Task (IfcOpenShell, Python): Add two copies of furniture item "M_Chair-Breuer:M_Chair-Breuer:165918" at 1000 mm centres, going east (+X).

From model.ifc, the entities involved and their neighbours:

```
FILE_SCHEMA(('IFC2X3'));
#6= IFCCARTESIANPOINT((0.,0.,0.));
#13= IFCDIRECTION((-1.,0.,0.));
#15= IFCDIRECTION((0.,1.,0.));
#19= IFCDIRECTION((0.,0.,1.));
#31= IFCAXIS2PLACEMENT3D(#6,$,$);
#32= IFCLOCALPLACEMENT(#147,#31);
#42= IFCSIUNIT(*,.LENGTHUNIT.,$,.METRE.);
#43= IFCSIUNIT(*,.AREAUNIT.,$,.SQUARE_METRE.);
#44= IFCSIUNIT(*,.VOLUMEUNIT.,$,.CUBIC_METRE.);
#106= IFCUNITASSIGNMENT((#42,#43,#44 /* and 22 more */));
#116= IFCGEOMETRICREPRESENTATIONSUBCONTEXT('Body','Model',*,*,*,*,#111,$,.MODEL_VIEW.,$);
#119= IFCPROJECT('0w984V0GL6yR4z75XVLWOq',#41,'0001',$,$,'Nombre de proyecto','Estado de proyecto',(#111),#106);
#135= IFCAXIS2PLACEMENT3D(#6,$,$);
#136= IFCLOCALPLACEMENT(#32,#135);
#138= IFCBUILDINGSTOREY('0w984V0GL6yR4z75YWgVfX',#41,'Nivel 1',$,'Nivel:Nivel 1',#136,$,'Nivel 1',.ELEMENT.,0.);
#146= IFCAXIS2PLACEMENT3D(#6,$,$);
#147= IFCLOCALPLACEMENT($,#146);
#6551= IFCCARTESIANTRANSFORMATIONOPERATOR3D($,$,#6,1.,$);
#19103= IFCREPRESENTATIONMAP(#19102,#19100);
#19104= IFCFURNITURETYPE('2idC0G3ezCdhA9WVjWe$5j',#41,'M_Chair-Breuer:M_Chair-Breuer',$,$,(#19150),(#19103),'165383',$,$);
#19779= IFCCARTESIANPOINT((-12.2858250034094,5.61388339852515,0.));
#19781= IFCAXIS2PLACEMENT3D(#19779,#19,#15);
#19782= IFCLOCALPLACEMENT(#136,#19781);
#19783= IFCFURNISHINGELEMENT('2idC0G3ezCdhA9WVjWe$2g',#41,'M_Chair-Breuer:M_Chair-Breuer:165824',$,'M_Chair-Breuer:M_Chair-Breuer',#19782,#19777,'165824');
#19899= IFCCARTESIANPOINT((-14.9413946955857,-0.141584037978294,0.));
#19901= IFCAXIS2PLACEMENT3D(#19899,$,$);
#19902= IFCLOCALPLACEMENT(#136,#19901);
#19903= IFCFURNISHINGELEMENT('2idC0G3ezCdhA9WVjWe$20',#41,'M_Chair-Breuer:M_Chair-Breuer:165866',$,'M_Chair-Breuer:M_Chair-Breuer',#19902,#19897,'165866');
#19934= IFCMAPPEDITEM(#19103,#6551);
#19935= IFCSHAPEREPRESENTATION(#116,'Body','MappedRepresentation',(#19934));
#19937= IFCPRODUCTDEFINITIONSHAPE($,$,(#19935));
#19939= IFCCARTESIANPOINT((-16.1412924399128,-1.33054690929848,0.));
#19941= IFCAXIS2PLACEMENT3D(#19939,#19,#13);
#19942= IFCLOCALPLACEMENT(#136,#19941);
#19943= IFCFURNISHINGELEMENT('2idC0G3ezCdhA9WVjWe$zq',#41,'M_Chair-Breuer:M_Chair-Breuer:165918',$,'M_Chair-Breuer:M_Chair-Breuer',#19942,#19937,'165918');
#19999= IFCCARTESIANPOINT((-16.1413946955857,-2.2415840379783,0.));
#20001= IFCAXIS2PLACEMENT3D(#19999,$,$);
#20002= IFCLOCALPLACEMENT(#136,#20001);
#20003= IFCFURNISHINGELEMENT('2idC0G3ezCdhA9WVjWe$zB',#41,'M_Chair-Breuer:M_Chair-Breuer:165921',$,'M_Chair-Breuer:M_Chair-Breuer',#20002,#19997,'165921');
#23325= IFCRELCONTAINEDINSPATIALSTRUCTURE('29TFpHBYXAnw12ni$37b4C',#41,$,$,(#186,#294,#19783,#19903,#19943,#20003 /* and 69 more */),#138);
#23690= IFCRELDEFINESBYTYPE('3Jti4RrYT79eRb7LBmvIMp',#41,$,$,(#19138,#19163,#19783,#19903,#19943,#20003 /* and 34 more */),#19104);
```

```python
import numpy as np
import ifcopenshell
import ifcopenshell.api.geometry
import ifcopenshell.api.root
import ifcopenshell.util.element
import ifcopenshell.util.placement
import ifcopenshell.util.unit

model = ifcopenshell.open("model.ifc")
unit_scale = ifcopenshell.util.unit.calculate_unit_scale(model)


def reuse_history(source, copy):
    """copy_class also copies each property set's owner history, people and application; keep the originals."""
    for rel in copy.IsDefinedBy:
        if rel.is_a("IfcRelDefinesByProperties") and (history := rel.RelatingPropertyDefinition.OwnerHistory):
            rel.RelatingPropertyDefinition.OwnerHistory = source.OwnerHistory
            ifcopenshell.util.element.remove_deep2(model, history)


source = model.by_guid("2idC0G3ezCdhA9WVjWe$zq")
base = ifcopenshell.util.placement.get_local_placement(source.ObjectPlacement)
step = np.array([1.0, 0.0, 0.0]) * 1 / unit_scale

for i in range(1, 3):
    copy = ifcopenshell.api.root.copy_class(model, product=source)
    copy.Representation = ifcopenshell.util.element.copy_deep(
        model, source.Representation, exclude=["IfcGeometricRepresentationContext", "IfcRepresentationMap"]
    )
    copy.Name = "M_Chair-Breuer:M_Chair-Breuer"
    copy.Tag = None
    reuse_history(source, copy)
    matrix = base.copy()
    matrix[:3, 3] += i * step
    print("added at", matrix[:3, 3].round(3) + 0.0)
    ifcopenshell.api.geometry.edit_object_placement(model, product=copy, matrix=matrix, is_si=False)

model.write("model-out.ifc")
```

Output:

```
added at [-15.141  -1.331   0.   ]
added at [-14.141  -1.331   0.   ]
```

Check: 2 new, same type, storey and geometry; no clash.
